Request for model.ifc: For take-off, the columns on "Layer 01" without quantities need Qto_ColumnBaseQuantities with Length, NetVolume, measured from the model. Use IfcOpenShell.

First a look at what the model holds.

```python
import ifcopenshell
import ifcopenshell.util.element
import ifcopenshell.util.unit

model = ifcopenshell.open("model.ifc")
print(model.schema)
for unit_type in ("LENGTHUNIT", "AREAUNIT", "VOLUMEUNIT"):
    print(unit_type, ifcopenshell.util.unit.calculate_unit_scale(model, unit_type))
storey = next(s for s in model.by_type("IfcBuildingStorey") if s.Name == "Layer 01")
columns = [e for e in ifcopenshell.util.element.get_decomposition(storey) if e.is_a("IfcColumn")]
for e in sorted(columns, key=lambda e: e.id()):
    print(e.id(), e.is_a(), e.Name, list(ifcopenshell.util.element.get_psets(e, qtos_only=True)), sep=" | ")
```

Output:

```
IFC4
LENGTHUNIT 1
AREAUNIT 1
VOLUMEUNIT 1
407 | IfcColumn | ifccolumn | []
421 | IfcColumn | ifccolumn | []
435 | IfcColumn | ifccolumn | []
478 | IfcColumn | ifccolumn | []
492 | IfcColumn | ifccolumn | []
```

```python
import ifcopenshell
import ifcopenshell.api.pset
import ifcopenshell.geom
import ifcopenshell.util.element
import ifcopenshell.util.shape
import ifcopenshell.util.unit

model = ifcopenshell.open("model.ifc")
unit_scale = ifcopenshell.util.unit.calculate_unit_scale(model)
volume_scale = ifcopenshell.util.unit.calculate_unit_scale(model, "VOLUMEUNIT")
settings = ifcopenshell.geom.settings()

storey = next(s for s in model.by_type("IfcBuildingStorey") if s.Name == "Layer 01")
columns = [e for e in ifcopenshell.util.element.get_decomposition(storey) if e.is_a("IfcColumn")]

for e in sorted(columns, key=lambda e: e.id()):
    if ifcopenshell.util.element.get_psets(e, qtos_only=True, should_inherit=False):
        continue
    # Geometry comes back in metres, in the element's own axes.
    shape = ifcopenshell.geom.create_shape(settings, e)
    values = {
        "Length": ifcopenshell.util.shape.get_z(shape.geometry) / unit_scale,
        "NetVolume": ifcopenshell.util.shape.get_volume(shape.geometry) / volume_scale,
    }
    qto = ifcopenshell.api.pset.add_qto(model, product=e, name="Qto_ColumnBaseQuantities")
    ifcopenshell.api.pset.edit_qto(model, qto=qto, properties=values)
    print(e.id(), {k: round(v, 3) for k, v in values.items()})

model.write("model_updated.ifc")
```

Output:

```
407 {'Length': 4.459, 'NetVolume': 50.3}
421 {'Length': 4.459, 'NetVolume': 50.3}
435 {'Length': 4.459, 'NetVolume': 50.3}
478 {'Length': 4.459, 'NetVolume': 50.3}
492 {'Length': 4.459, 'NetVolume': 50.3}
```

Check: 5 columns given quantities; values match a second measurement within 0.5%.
